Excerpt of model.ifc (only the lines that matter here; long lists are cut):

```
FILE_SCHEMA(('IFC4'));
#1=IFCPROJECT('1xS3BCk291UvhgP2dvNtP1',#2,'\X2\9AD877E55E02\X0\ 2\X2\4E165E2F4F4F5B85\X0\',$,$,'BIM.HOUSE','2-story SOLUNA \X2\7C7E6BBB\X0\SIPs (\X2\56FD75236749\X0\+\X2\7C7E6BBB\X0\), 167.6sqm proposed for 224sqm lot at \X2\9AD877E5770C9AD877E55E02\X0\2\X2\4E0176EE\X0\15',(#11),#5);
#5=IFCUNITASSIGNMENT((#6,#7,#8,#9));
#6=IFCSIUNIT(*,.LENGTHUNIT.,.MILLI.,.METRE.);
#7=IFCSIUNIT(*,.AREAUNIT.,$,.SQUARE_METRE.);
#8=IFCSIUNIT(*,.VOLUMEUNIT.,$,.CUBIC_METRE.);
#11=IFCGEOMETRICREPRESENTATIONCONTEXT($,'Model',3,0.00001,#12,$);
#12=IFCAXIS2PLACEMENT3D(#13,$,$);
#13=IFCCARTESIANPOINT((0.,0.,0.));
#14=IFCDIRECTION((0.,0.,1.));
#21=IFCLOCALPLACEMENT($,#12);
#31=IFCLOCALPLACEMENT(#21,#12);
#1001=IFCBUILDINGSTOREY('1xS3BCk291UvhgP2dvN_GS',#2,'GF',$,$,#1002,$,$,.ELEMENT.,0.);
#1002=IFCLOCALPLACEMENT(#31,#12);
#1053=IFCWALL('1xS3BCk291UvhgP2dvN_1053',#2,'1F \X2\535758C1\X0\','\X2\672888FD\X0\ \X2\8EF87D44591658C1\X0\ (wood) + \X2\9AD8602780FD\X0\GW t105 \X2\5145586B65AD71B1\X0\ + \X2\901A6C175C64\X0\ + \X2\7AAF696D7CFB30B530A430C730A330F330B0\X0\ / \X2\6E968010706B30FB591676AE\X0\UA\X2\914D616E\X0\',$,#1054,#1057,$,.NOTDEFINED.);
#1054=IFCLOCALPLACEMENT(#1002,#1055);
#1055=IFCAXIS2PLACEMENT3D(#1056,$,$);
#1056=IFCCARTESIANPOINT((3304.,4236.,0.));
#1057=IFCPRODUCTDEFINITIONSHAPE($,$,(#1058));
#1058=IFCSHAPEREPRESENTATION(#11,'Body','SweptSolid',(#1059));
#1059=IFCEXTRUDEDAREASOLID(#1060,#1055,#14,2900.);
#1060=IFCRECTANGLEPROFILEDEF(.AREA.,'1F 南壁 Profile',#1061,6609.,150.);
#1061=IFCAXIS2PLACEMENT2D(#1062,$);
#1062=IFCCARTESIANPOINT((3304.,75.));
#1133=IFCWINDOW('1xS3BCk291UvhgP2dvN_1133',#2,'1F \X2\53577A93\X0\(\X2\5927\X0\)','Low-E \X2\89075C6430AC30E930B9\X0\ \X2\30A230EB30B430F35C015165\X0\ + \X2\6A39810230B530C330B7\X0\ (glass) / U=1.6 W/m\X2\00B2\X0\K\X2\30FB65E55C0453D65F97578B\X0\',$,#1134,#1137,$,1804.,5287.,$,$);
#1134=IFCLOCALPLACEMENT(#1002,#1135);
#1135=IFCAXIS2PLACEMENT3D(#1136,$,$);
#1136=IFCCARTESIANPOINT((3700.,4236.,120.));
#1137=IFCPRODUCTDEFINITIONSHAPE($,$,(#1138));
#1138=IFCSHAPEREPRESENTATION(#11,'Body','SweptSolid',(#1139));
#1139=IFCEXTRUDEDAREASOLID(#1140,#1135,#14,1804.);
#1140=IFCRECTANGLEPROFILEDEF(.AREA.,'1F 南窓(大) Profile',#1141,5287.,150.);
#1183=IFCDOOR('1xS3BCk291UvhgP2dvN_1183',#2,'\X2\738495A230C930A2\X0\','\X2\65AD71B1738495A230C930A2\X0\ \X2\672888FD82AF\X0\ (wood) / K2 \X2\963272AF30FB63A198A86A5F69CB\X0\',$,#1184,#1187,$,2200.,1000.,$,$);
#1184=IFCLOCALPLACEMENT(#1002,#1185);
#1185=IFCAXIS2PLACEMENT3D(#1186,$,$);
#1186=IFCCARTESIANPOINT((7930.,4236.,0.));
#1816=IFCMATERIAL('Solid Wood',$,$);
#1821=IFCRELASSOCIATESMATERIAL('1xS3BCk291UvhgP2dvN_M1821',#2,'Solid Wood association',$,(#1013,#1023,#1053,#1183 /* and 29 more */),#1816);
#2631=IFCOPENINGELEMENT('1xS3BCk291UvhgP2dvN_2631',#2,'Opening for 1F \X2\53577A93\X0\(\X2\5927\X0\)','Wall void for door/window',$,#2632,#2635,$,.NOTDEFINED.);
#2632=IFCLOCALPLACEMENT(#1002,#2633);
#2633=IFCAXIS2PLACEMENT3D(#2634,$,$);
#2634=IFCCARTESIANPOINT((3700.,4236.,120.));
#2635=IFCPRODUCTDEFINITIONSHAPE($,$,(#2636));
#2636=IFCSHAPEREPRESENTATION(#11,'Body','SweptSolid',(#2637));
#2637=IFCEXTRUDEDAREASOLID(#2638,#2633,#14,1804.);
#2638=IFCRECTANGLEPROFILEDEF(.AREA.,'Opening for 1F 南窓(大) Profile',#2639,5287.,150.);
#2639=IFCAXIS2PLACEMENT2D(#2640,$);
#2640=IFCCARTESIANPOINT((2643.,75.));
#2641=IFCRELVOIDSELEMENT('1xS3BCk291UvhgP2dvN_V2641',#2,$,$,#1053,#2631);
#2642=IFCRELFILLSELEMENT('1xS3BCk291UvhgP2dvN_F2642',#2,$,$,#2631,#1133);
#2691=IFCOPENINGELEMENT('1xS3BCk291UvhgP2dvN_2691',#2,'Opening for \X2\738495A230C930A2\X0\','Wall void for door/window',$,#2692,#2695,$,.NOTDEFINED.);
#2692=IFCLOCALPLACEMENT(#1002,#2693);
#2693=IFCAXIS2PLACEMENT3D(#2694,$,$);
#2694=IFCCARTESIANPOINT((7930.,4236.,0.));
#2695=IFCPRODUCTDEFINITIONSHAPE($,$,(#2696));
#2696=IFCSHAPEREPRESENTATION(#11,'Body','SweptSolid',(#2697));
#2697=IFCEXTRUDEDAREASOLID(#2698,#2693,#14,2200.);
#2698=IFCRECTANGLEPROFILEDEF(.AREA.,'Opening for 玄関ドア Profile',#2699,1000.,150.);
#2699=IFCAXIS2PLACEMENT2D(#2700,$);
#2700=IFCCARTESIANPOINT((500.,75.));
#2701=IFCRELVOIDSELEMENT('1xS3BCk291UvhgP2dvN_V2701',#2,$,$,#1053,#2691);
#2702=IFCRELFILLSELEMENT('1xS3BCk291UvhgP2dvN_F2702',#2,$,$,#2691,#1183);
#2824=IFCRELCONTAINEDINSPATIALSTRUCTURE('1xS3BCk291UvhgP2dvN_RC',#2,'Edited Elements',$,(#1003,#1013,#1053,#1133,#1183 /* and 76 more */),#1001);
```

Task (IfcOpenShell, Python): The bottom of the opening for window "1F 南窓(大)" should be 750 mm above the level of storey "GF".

```python
import numpy as np
import ifcopenshell
import ifcopenshell.api.geometry
import ifcopenshell.geom
import ifcopenshell.util.element
import ifcopenshell.util.placement
import ifcopenshell.util.shape
import ifcopenshell.util.unit

model = ifcopenshell.open("model.ifc")
unit_scale = ifcopenshell.util.unit.calculate_unit_scale(model)

window = model.by_id(1133)
opening = window.FillsVoids[0].RelatingOpeningElement
storey = ifcopenshell.util.element.get_container(window, ifc_class="IfcBuildingStorey")
level = ifcopenshell.util.placement.get_local_placement(storey.ObjectPlacement)[2, 3]

# The opening's origin need not be at the sill, so measure its lowest point.
shape = ifcopenshell.geom.create_shape(ifcopenshell.geom.settings(), opening)
bottom = ifcopenshell.util.shape.get_shape_bottom_elevation(shape, shape.geometry) / unit_scale
dz = level + 0.75 / unit_scale - bottom

shift = np.array([0.0, 0.0, dz])
# The window is not placed relative to its opening, so move both.
for product in (opening, window):
    matrix = ifcopenshell.util.placement.get_local_placement(product.ObjectPlacement)
    matrix[:3, 3] += shift
    ifcopenshell.api.geometry.edit_object_placement(model, product=product, matrix=matrix, is_si=False)

print(f"moved by {dz * unit_scale:+.3f} m")

model.write("model_updated.ifc")
```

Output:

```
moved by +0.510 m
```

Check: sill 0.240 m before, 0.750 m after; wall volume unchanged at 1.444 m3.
